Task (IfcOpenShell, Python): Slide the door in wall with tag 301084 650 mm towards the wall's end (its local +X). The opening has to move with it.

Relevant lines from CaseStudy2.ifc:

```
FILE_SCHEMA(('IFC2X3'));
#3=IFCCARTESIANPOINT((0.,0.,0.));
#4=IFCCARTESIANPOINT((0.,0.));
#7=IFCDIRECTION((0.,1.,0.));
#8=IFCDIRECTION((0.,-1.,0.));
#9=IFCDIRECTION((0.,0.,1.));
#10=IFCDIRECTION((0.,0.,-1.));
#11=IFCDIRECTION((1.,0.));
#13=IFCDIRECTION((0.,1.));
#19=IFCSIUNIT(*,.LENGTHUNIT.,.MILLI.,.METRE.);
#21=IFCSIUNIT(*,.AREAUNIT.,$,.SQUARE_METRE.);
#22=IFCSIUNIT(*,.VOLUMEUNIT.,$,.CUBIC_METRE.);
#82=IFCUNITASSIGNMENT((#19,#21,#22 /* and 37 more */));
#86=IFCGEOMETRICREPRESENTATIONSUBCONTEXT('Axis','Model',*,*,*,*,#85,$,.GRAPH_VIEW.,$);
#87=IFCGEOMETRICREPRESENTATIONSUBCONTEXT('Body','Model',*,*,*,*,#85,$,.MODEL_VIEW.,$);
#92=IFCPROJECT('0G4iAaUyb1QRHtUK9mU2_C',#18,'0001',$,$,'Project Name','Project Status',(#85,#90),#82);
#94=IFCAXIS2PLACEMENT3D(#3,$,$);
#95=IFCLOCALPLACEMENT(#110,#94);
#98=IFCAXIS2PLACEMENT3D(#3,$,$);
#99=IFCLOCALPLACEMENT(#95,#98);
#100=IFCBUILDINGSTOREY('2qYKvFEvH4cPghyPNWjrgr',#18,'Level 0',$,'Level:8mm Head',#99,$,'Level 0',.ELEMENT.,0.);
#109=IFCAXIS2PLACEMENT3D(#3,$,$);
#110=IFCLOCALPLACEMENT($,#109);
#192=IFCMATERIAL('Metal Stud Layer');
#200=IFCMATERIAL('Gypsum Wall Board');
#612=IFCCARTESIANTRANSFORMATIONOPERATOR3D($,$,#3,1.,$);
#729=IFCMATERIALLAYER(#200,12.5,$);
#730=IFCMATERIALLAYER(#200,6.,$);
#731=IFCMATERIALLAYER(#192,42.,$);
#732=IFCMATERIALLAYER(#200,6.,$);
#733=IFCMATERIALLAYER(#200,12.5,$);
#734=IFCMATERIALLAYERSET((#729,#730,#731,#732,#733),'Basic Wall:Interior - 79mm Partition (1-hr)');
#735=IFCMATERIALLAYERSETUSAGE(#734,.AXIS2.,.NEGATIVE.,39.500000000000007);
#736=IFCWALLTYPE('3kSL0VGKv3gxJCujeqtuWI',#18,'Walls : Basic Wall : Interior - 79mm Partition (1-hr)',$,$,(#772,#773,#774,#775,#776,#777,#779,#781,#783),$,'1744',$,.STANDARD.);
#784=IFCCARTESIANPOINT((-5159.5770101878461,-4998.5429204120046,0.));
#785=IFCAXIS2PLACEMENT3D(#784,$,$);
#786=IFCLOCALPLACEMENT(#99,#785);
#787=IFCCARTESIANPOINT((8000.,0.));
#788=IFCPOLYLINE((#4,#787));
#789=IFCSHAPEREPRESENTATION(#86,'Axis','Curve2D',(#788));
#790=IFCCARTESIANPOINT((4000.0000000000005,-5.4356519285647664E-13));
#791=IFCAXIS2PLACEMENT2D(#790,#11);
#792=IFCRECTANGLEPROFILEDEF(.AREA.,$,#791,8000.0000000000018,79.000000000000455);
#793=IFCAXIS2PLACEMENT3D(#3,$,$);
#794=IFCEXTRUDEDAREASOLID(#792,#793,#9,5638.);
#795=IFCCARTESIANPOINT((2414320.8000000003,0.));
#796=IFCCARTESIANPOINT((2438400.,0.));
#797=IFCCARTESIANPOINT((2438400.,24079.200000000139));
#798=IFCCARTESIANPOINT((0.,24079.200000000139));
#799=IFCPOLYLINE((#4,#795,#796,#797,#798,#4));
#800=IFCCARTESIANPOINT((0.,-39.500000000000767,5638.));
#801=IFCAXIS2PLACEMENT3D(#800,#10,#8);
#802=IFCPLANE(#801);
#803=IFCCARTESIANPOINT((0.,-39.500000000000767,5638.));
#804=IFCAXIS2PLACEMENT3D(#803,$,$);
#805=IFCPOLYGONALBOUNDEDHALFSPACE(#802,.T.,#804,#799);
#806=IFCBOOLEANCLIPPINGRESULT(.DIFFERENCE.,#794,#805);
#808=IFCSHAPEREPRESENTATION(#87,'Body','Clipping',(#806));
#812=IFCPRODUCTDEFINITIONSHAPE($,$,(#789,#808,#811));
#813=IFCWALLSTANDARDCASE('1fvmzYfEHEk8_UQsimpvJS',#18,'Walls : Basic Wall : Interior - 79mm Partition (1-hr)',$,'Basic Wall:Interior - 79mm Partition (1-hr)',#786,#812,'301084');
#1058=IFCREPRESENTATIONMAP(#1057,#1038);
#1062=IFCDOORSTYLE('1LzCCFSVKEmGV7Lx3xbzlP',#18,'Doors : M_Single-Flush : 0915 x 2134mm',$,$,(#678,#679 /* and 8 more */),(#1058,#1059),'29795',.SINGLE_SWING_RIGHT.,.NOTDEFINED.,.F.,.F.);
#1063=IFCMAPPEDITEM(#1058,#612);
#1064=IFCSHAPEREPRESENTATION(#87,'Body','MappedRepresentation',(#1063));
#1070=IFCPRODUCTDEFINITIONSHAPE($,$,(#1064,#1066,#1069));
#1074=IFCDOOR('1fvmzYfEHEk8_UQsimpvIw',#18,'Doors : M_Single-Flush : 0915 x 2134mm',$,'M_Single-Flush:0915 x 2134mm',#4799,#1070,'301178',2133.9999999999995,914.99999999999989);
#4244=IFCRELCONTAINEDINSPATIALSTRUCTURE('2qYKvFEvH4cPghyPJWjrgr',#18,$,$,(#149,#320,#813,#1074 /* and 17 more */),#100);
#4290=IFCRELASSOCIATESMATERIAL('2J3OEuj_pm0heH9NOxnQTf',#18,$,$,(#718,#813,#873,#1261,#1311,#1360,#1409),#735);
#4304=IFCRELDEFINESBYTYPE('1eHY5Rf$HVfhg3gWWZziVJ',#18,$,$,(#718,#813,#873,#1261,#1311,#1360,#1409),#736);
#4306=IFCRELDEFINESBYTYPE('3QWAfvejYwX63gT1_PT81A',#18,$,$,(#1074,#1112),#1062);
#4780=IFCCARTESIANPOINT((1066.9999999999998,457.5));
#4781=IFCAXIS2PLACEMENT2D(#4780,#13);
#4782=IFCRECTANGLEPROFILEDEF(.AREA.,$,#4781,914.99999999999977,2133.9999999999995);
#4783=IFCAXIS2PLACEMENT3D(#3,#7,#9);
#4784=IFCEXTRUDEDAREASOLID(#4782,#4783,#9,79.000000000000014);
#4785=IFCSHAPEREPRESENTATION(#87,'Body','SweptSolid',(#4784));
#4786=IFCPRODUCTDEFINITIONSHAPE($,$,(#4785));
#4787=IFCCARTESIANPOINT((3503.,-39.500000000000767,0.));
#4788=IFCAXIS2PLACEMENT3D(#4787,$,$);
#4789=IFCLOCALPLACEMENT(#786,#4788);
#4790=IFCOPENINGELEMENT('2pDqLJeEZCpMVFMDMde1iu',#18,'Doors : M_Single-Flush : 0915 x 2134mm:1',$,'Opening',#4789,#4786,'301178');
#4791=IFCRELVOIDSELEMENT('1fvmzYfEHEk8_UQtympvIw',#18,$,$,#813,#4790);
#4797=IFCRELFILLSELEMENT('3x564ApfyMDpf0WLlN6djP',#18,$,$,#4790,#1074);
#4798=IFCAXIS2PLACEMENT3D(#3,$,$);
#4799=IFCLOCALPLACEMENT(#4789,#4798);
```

```python
import ifcopenshell
import ifcopenshell.api.geometry
import ifcopenshell.util.placement
import ifcopenshell.util.unit

model = ifcopenshell.open("CaseStudy2.ifc")
unit_scale = ifcopenshell.util.unit.calculate_unit_scale(model)

door = model.by_guid("1fvmzYfEHEk8_UQsimpvIw")
opening = door.FillsVoids[0].RelatingOpeningElement
wall = opening.VoidsElements[0].RelatingBuildingElement

wall_matrix = ifcopenshell.util.placement.get_local_placement(wall.ObjectPlacement)
shift = wall_matrix[:3, 0] * 0.65 / unit_scale
before = ifcopenshell.util.placement.get_local_placement(door.ObjectPlacement)[:3, 3].copy()

# The door is placed relative to its opening, so it follows when the opening moves.
matrix = ifcopenshell.util.placement.get_local_placement(opening.ObjectPlacement)
matrix[:3, 3] += shift
ifcopenshell.api.geometry.edit_object_placement(
    model, product=opening, matrix=matrix, is_si=False, should_transform_children=True
)

after = ifcopenshell.util.placement.get_local_placement(door.ObjectPlacement)[:3, 3]
print("door moved by", (after - before).round(3) + 0.0)

model.write("CaseStudy2-out.ifc")
```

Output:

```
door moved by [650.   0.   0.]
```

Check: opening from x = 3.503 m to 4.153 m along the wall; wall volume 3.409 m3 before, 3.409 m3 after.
